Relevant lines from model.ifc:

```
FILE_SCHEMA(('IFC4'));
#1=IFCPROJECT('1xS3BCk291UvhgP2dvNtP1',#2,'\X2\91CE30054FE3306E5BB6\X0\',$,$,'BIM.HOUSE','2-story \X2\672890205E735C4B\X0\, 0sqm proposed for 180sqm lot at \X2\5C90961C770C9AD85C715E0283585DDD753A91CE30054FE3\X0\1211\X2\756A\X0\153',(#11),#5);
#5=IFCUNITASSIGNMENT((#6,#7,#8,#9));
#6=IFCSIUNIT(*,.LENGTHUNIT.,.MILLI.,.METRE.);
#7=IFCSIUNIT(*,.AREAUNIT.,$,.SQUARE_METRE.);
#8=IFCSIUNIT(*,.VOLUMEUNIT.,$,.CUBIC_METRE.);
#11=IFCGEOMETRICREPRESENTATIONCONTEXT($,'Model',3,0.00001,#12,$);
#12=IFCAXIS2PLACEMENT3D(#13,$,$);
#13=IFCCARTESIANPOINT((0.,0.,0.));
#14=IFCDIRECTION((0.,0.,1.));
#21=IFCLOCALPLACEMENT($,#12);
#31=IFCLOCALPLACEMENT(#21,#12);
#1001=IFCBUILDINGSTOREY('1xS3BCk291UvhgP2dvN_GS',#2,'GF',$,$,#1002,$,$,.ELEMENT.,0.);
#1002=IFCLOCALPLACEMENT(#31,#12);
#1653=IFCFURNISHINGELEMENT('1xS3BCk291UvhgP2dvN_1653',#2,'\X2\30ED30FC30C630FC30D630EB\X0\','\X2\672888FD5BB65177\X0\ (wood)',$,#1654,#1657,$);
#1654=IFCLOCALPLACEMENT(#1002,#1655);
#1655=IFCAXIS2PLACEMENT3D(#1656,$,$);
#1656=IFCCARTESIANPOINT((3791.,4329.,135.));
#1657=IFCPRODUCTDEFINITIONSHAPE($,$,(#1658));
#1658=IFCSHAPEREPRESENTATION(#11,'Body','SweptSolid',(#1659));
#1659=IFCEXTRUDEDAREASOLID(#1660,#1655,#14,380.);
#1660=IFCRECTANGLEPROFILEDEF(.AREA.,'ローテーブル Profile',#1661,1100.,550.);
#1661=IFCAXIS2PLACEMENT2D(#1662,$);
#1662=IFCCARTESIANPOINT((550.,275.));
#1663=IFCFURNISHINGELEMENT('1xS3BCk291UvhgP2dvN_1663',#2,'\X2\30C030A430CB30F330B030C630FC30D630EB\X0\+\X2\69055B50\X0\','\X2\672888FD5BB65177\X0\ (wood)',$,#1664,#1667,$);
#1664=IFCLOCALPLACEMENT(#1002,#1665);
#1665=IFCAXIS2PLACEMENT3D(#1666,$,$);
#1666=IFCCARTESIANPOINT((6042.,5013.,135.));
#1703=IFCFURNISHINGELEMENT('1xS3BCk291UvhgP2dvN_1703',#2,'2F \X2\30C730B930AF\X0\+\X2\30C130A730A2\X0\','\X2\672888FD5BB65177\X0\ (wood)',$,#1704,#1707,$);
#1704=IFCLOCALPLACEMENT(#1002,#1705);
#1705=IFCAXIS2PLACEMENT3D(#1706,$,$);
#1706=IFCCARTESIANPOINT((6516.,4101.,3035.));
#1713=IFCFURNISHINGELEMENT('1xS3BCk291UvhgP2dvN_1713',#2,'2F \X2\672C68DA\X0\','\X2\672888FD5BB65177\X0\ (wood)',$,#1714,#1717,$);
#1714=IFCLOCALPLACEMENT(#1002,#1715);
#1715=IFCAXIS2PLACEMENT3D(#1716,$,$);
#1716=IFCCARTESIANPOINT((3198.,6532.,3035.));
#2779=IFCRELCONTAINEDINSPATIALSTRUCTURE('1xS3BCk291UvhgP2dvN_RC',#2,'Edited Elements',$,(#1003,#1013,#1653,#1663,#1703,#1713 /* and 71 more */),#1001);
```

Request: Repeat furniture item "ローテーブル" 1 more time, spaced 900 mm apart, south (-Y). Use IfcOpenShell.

```python
import numpy as np
import ifcopenshell
import ifcopenshell.api.geometry
import ifcopenshell.api.root
import ifcopenshell.util.element
import ifcopenshell.util.placement
import ifcopenshell.util.unit

model = ifcopenshell.open("model.ifc")
unit_scale = ifcopenshell.util.unit.calculate_unit_scale(model)


def reuse_history(source, copy):
    """copy_class also copies each property set's owner history, people and application; keep the originals."""
    for rel in copy.IsDefinedBy:
        if rel.is_a("IfcRelDefinesByProperties") and (history := rel.RelatingPropertyDefinition.OwnerHistory):
            rel.RelatingPropertyDefinition.OwnerHistory = source.OwnerHistory
            ifcopenshell.util.element.remove_deep2(model, history)


source = model.by_guid("1xS3BCk291UvhgP2dvN_1653")
base = ifcopenshell.util.placement.get_local_placement(source.ObjectPlacement)
step = np.array([0.0, -1.0, 0.0]) * 0.9 / unit_scale

for i in range(1, 2):
    copy = ifcopenshell.api.root.copy_class(model, product=source)
    copy.Representation = ifcopenshell.util.element.copy_deep(
        model, source.Representation, exclude=["IfcGeometricRepresentationContext", "IfcRepresentationMap"]
    )
    reuse_history(source, copy)
    matrix = base.copy()
    matrix[:3, 3] += i * step
    print("added at", matrix[:3, 3].round(3) + 0.0)
    ifcopenshell.api.geometry.edit_object_placement(model, product=copy, matrix=matrix, is_si=False)

model.write("model_rev.ifc")
```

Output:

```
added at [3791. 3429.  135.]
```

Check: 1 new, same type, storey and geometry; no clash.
